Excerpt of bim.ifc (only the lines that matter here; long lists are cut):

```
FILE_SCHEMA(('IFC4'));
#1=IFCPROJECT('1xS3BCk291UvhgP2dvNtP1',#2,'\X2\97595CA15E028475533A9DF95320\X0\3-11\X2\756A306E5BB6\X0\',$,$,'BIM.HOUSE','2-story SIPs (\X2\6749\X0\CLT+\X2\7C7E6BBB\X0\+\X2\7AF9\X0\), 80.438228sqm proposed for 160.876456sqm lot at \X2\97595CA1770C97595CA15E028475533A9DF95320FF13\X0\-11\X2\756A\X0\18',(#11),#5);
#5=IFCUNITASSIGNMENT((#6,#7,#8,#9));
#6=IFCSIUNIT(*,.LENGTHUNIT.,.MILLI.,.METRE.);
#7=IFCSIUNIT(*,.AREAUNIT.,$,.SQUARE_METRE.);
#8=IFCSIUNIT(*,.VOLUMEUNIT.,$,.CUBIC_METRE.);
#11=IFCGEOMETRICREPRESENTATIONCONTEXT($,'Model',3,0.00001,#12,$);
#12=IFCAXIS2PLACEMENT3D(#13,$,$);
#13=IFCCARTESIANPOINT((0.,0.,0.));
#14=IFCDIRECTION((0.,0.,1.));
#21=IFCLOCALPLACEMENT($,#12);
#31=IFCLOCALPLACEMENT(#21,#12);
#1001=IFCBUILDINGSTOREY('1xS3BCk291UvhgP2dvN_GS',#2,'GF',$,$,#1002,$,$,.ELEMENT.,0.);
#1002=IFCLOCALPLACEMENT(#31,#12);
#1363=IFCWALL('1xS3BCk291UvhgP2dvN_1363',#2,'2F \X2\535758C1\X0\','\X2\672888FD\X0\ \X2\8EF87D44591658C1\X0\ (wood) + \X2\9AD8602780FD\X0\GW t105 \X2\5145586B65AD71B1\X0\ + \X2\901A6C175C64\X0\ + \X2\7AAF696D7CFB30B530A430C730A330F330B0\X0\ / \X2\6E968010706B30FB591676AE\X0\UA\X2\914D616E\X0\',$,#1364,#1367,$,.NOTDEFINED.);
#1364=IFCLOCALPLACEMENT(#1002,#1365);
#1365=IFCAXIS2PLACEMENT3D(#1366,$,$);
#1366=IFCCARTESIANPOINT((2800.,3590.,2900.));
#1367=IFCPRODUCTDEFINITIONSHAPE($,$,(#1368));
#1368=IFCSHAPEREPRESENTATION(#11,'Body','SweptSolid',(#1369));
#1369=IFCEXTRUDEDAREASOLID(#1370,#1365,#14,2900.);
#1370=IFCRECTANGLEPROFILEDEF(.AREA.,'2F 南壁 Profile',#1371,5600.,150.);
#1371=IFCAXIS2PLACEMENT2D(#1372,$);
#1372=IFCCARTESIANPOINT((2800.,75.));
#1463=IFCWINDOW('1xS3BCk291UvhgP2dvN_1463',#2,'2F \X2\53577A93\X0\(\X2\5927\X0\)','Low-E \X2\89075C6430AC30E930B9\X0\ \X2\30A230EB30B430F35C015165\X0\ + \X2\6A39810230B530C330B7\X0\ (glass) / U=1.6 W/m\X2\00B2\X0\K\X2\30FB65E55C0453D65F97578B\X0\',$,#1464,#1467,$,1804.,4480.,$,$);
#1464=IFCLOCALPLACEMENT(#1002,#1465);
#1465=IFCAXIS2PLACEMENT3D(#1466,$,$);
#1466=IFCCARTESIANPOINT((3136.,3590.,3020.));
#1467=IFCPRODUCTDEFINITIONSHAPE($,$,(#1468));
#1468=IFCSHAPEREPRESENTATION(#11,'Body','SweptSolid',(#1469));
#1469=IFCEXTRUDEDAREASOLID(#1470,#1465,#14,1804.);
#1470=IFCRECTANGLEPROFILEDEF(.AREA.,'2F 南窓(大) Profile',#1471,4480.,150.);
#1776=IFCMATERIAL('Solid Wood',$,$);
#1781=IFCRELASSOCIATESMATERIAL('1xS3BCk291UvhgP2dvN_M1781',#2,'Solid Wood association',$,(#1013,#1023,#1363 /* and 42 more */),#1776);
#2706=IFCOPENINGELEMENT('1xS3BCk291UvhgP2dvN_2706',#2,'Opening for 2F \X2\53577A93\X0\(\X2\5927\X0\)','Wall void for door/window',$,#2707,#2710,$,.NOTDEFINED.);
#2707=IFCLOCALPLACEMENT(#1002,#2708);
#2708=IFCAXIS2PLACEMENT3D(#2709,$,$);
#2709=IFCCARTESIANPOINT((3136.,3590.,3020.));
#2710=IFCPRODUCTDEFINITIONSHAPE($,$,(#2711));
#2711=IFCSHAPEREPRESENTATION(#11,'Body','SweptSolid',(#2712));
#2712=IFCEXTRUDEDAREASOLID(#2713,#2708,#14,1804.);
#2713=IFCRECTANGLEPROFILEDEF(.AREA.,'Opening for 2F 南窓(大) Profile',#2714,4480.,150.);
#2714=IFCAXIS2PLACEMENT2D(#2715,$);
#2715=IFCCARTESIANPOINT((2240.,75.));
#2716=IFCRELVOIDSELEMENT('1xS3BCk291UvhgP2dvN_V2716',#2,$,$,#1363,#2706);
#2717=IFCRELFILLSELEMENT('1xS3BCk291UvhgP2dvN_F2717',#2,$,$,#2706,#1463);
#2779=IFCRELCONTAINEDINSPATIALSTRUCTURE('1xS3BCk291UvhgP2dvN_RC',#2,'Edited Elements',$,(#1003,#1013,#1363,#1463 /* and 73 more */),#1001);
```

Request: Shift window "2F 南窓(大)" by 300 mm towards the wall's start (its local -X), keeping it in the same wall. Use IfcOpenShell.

```python
import ifcopenshell
import ifcopenshell.api.geometry
import ifcopenshell.util.placement
import ifcopenshell.util.unit

model = ifcopenshell.open("bim.ifc")
unit_scale = ifcopenshell.util.unit.calculate_unit_scale(model)

window = model.by_id(1463)
opening = window.FillsVoids[0].RelatingOpeningElement
wall = opening.VoidsElements[0].RelatingBuildingElement

wall_matrix = ifcopenshell.util.placement.get_local_placement(wall.ObjectPlacement)
shift = wall_matrix[:3, 0] * -0.3 / unit_scale
before = ifcopenshell.util.placement.get_local_placement(window.ObjectPlacement)[:3, 3].copy()

# The window is not placed relative to its opening, so move both.
for product in (opening, window):
    matrix = ifcopenshell.util.placement.get_local_placement(product.ObjectPlacement)
    matrix[:3, 3] += shift
    ifcopenshell.api.geometry.edit_object_placement(model, product=product, matrix=matrix, is_si=False)

after = ifcopenshell.util.placement.get_local_placement(window.ObjectPlacement)[:3, 3]
print("window moved by", (after - before).round(3) + 0.0)

model.write("bim_edited.ifc")
```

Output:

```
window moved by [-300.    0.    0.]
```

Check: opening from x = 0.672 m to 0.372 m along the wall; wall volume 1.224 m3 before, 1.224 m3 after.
